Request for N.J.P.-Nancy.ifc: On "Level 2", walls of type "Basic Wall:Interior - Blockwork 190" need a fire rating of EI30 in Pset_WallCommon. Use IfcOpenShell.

First a look at what the model holds.

```python
import ifcopenshell
import ifcopenshell.util.element

model = ifcopenshell.open("N.J.P.-Nancy.ifc")
print(model.schema)
storey = next(s for s in model.by_type("IfcBuildingStorey") if s.Name == "Level 2")
walls = [e for e in ifcopenshell.util.element.get_decomposition(storey) if e.is_a("IfcWall")]
seen = {}
for e in walls:
    element_type = ifcopenshell.util.element.get_type(e)
    key = (element_type.Name if element_type != e and element_type else None, ifcopenshell.util.element.get_pset(e, "Pset_WallCommon", "FireRating"))
    seen[key] = seen.get(key, 0) + 1
for (name, value), count in sorted(seen.items(), key=str):
    print(count, "x", name, "|", value)
```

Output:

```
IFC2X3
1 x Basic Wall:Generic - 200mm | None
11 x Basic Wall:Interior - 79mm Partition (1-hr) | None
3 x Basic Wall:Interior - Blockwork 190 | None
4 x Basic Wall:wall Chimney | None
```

```python
import ifcopenshell
import ifcopenshell.api.pset
import ifcopenshell.util.element

model = ifcopenshell.open("N.J.P.-Nancy.ifc")

storey = next(s for s in model.by_type("IfcBuildingStorey") if s.Name == "Level 2")
walls = [e for e in ifcopenshell.util.element.get_decomposition(storey) if e.is_a("IfcWall")]

count = 0
for e in walls:
    element_type = ifcopenshell.util.element.get_type(e)
    if element_type in (None, e) or element_type.Name != "Basic Wall:Interior - Blockwork 190":
        continue
    # add_pset returns the element's existing set when there is one.
    pset = ifcopenshell.api.pset.add_pset(model, product=e, name="Pset_WallCommon")
    ifcopenshell.api.pset.edit_pset(model, pset=pset, properties={"FireRating": "EI30"})
    count += 1

print(count, "walls updated")

model.write("N.J.P.-Nancy_rev.ifc")
```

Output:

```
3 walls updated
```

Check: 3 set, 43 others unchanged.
